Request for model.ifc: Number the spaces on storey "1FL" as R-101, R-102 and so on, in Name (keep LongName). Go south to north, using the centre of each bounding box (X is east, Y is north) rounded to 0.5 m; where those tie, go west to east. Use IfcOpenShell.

First a look at what the model holds.

```python
import ifcopenshell
import ifcopenshell.util.element
import ifcopenshell.util.placement

model = ifcopenshell.open("model.ifc")
print(model.schema)
storey = next(s for s in model.by_type("IfcBuildingStorey") if s.Name == "1FL")
spaces = [e for e in ifcopenshell.util.element.get_decomposition(storey) if e.is_a("IfcSpace")]
for e in sorted(spaces, key=lambda e: e.id()):
    origin = ifcopenshell.util.placement.get_local_placement(e.ObjectPlacement)[:3, 3]
    print(e.id(), e.Name, e.LongName, origin.round(2) + 0.0, sep=" | ")
```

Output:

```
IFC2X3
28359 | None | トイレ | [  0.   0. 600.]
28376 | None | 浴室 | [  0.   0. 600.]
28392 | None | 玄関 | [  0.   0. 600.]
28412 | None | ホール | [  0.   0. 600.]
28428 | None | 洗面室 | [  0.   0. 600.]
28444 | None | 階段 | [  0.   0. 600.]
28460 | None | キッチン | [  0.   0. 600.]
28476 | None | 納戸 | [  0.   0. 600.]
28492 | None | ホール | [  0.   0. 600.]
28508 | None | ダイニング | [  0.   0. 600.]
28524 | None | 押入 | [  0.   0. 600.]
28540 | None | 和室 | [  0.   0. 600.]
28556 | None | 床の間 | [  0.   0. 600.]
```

```python
import ifcopenshell
import ifcopenshell.geom
import ifcopenshell.util.element
import ifcopenshell.util.shape

model = ifcopenshell.open("model.ifc")
settings = ifcopenshell.geom.settings()
settings.set("use-world-coords", True)


def centre(element):
    shape = ifcopenshell.geom.create_shape(settings, element)
    return ifcopenshell.util.shape.get_bbox_centroid(shape.geometry)


storey = next(s for s in model.by_type("IfcBuildingStorey") if s.Name == "1FL")
spaces = [e for e in ifcopenshell.util.element.get_decomposition(storey) if e.is_a("IfcSpace")]

# Insertion points can sit at a corner or the storey origin, so sort by the geometry (in metres).
centres = {e: centre(e) for e in spaces}
spaces.sort(key=lambda e: (round(centres[e][1] / 0.5), centres[e][0]))

for i, e in enumerate(spaces, start=1):
    number = f"R-1{i:02d}"
    e.Name = number
    print(e.id(), number)

model.write("model_updated.ifc")
```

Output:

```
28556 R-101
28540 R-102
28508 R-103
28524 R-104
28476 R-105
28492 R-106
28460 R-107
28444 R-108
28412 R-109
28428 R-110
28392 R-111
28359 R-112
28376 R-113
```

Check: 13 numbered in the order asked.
